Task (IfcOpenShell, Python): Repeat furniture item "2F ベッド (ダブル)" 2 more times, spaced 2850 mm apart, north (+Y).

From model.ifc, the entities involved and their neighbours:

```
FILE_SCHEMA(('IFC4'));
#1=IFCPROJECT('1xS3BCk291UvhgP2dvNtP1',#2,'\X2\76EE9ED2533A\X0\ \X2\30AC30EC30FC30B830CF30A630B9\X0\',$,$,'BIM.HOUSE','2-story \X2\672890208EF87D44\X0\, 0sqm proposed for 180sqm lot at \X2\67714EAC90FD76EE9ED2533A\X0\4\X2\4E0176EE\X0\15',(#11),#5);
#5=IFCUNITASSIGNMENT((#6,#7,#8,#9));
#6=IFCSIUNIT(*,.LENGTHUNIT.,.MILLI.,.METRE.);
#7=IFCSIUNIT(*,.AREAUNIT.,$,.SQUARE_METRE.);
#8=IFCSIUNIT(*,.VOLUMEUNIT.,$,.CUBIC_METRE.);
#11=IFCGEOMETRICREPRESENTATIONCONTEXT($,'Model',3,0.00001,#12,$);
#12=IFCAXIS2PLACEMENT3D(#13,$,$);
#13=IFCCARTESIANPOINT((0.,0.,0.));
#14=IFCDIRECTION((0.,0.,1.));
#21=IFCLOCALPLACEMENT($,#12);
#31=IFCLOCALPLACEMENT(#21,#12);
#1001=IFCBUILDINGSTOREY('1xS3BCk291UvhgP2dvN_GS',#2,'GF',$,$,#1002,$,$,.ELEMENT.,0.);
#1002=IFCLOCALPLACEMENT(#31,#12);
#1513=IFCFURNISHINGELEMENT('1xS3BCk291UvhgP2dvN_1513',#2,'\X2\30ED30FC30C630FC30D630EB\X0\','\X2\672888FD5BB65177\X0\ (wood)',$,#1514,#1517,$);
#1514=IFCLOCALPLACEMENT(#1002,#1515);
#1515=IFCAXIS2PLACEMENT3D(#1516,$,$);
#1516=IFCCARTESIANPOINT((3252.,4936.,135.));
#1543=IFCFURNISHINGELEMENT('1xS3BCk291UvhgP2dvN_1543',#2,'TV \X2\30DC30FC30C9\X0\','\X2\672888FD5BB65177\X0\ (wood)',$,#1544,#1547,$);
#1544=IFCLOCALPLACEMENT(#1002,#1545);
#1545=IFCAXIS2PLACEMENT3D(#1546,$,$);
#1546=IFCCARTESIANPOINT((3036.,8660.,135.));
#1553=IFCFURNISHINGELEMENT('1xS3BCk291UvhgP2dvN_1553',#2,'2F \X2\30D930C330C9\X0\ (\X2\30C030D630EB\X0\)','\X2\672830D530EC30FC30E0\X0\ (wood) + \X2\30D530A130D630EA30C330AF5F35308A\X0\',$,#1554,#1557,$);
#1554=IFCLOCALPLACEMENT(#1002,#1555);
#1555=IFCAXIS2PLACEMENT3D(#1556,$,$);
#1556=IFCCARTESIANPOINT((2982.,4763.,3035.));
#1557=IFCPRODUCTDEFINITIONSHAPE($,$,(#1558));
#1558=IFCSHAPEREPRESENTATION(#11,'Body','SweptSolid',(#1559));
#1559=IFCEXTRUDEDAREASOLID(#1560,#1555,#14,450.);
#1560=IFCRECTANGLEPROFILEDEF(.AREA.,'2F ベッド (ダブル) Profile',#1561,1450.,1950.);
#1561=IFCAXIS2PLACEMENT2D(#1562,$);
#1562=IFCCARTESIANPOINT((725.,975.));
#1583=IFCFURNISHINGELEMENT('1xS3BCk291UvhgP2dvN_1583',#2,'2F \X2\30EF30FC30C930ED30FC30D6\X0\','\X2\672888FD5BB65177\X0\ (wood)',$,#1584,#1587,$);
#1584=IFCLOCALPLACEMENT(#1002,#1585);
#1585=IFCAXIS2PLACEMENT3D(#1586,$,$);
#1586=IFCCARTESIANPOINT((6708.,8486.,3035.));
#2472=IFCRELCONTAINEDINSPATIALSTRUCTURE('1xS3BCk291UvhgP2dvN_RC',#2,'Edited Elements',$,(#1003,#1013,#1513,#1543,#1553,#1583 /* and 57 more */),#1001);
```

```python
import numpy as np
import ifcopenshell
import ifcopenshell.api.geometry
import ifcopenshell.api.root
import ifcopenshell.util.element
import ifcopenshell.util.placement

model = ifcopenshell.open("model.ifc")


def reuse_history(source, copy):
    """copy_class also copies each property set's owner history, people and application; keep the originals."""
    for rel in copy.IsDefinedBy:
        if rel.is_a("IfcRelDefinesByProperties") and (history := rel.RelatingPropertyDefinition.OwnerHistory):
            rel.RelatingPropertyDefinition.OwnerHistory = source.OwnerHistory
            ifcopenshell.util.element.remove_deep2(model, history)


source = model.by_guid("1xS3BCk291UvhgP2dvN_1553")
base = ifcopenshell.util.placement.get_local_placement(source.ObjectPlacement)
step = np.array([0.0, 1.0, 0.0]) * 2850.0

for i in range(1, 3):
    copy = ifcopenshell.api.root.copy_class(model, product=source)
    copy.Representation = ifcopenshell.util.element.copy_deep(
        model, source.Representation, exclude=["IfcGeometricRepresentationContext", "IfcRepresentationMap"]
    )
    reuse_history(source, copy)
    matrix = base.copy()
    matrix[:3, 3] += i * step
    print("added at", matrix[:3, 3].round(3) + 0.0)
    ifcopenshell.api.geometry.edit_object_placement(model, product=copy, matrix=matrix, is_si=False)

model.write("model_rev.ifc")
```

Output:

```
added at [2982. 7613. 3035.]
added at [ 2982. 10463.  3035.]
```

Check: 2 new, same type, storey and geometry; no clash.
